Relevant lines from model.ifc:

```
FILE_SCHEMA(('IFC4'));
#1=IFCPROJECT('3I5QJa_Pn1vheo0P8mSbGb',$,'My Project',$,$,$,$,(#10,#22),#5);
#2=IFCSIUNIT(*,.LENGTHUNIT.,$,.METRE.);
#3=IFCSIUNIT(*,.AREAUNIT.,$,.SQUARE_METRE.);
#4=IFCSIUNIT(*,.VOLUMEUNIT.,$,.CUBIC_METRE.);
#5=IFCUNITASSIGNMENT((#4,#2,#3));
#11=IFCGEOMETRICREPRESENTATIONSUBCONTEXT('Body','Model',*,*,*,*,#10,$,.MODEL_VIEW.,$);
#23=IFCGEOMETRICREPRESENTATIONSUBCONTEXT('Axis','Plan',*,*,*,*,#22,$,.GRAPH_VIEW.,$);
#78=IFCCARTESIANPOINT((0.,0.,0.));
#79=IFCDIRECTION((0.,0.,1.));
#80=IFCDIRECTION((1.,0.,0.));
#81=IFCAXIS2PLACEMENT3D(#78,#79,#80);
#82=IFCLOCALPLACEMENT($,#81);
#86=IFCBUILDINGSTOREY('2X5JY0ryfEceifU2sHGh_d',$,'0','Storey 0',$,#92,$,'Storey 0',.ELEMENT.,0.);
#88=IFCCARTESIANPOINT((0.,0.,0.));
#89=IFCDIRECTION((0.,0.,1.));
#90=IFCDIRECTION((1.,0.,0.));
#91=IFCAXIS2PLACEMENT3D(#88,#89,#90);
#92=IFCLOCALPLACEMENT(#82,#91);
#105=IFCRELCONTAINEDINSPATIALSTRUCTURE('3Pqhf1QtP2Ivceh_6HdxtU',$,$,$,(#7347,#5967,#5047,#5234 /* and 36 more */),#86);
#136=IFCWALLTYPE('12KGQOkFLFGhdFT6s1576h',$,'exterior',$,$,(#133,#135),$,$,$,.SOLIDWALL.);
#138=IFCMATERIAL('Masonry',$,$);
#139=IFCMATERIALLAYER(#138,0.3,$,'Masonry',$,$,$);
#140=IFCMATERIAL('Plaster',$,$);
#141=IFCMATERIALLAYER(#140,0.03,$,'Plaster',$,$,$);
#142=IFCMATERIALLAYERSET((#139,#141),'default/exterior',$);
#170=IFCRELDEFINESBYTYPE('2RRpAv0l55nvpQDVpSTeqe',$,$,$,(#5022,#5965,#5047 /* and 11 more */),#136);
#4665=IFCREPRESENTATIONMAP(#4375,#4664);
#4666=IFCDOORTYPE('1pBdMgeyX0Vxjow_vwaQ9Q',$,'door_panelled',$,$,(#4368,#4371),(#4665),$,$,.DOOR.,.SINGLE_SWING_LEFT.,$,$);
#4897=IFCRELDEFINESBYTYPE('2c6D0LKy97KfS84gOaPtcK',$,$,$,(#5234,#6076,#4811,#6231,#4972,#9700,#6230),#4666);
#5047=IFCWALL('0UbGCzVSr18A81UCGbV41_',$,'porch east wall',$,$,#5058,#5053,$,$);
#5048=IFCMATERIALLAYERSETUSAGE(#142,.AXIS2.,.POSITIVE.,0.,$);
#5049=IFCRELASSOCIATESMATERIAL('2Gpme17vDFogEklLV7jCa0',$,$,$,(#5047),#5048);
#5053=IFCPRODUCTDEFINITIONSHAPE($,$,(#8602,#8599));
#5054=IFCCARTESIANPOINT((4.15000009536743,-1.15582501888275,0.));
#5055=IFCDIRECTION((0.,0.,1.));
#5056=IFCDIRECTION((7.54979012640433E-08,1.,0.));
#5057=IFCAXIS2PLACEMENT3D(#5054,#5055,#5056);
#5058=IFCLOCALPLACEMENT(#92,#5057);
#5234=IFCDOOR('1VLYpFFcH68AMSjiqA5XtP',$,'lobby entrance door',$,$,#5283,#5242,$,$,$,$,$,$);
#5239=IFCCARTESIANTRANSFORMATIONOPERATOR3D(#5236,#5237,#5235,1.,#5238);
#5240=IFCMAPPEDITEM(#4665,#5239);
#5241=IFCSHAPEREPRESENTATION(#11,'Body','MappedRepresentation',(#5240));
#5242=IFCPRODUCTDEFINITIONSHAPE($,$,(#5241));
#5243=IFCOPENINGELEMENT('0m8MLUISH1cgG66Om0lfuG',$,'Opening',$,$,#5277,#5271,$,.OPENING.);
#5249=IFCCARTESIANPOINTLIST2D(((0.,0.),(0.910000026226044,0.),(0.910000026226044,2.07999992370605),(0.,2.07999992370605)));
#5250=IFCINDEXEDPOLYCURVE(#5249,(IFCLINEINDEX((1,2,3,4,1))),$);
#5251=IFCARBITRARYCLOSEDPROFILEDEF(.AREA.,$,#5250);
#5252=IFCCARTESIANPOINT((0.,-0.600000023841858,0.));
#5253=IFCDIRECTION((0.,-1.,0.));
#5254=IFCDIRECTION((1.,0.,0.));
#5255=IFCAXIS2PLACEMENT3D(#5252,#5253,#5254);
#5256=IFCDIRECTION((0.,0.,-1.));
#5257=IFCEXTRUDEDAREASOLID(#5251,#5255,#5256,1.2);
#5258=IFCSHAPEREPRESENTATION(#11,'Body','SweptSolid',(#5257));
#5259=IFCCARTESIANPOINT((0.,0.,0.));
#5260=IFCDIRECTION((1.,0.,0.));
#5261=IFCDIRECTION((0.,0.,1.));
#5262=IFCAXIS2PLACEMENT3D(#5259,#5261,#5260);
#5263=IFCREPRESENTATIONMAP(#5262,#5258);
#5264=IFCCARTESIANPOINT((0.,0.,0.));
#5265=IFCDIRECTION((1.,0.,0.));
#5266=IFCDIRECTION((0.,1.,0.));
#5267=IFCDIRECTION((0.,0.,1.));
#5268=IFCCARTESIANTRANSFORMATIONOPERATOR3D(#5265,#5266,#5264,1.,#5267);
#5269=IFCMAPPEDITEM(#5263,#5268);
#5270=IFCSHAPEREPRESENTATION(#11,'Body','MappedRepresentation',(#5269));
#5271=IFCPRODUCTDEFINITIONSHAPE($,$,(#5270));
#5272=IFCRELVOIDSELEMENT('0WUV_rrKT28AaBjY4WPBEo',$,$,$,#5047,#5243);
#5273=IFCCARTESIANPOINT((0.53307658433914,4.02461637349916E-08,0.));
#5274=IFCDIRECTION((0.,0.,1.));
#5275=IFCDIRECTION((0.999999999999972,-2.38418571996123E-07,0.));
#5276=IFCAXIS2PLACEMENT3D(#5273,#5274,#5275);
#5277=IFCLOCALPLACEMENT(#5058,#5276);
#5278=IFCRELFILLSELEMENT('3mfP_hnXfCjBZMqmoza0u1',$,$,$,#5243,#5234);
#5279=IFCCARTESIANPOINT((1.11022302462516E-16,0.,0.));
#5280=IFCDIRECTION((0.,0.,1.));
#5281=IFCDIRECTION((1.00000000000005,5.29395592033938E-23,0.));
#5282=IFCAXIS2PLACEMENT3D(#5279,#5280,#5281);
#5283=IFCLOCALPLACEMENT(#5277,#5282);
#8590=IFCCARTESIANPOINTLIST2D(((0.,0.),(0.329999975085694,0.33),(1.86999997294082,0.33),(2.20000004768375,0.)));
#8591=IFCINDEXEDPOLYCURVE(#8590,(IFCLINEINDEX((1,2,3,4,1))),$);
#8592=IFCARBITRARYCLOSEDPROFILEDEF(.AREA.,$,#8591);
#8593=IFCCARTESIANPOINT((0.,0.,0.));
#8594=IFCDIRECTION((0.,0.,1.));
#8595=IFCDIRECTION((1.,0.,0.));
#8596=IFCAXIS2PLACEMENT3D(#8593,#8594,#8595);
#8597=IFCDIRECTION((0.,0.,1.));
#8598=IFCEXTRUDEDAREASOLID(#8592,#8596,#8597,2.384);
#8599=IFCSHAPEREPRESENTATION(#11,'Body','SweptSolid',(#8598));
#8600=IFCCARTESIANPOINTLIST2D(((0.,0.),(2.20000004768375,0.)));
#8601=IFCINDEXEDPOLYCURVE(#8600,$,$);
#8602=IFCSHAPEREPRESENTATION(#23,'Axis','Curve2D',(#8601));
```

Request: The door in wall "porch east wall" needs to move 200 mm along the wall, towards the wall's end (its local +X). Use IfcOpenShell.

```python
import ifcopenshell
import ifcopenshell.api.geometry
import ifcopenshell.util.placement
import ifcopenshell.util.unit

model = ifcopenshell.open("model.ifc")
unit_scale = ifcopenshell.util.unit.calculate_unit_scale(model)

door = model.by_guid("1VLYpFFcH68AMSjiqA5XtP")
opening = door.FillsVoids[0].RelatingOpeningElement
wall = opening.VoidsElements[0].RelatingBuildingElement

wall_matrix = ifcopenshell.util.placement.get_local_placement(wall.ObjectPlacement)
shift = wall_matrix[:3, 0] * 0.2 / unit_scale
before = ifcopenshell.util.placement.get_local_placement(door.ObjectPlacement)[:3, 3].copy()

# The door is placed relative to its opening, so it follows when the opening moves.
matrix = ifcopenshell.util.placement.get_local_placement(opening.ObjectPlacement)
matrix[:3, 3] += shift
ifcopenshell.api.geometry.edit_object_placement(
    model, product=opening, matrix=matrix, is_si=False, should_transform_children=True
)

after = ifcopenshell.util.placement.get_local_placement(door.ObjectPlacement)[:3, 3]
print("door moved by", (after - before).round(3) + 0.0)

model.write("model-out.ifc")
```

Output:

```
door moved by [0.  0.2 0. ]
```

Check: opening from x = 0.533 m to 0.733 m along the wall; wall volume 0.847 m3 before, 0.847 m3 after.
